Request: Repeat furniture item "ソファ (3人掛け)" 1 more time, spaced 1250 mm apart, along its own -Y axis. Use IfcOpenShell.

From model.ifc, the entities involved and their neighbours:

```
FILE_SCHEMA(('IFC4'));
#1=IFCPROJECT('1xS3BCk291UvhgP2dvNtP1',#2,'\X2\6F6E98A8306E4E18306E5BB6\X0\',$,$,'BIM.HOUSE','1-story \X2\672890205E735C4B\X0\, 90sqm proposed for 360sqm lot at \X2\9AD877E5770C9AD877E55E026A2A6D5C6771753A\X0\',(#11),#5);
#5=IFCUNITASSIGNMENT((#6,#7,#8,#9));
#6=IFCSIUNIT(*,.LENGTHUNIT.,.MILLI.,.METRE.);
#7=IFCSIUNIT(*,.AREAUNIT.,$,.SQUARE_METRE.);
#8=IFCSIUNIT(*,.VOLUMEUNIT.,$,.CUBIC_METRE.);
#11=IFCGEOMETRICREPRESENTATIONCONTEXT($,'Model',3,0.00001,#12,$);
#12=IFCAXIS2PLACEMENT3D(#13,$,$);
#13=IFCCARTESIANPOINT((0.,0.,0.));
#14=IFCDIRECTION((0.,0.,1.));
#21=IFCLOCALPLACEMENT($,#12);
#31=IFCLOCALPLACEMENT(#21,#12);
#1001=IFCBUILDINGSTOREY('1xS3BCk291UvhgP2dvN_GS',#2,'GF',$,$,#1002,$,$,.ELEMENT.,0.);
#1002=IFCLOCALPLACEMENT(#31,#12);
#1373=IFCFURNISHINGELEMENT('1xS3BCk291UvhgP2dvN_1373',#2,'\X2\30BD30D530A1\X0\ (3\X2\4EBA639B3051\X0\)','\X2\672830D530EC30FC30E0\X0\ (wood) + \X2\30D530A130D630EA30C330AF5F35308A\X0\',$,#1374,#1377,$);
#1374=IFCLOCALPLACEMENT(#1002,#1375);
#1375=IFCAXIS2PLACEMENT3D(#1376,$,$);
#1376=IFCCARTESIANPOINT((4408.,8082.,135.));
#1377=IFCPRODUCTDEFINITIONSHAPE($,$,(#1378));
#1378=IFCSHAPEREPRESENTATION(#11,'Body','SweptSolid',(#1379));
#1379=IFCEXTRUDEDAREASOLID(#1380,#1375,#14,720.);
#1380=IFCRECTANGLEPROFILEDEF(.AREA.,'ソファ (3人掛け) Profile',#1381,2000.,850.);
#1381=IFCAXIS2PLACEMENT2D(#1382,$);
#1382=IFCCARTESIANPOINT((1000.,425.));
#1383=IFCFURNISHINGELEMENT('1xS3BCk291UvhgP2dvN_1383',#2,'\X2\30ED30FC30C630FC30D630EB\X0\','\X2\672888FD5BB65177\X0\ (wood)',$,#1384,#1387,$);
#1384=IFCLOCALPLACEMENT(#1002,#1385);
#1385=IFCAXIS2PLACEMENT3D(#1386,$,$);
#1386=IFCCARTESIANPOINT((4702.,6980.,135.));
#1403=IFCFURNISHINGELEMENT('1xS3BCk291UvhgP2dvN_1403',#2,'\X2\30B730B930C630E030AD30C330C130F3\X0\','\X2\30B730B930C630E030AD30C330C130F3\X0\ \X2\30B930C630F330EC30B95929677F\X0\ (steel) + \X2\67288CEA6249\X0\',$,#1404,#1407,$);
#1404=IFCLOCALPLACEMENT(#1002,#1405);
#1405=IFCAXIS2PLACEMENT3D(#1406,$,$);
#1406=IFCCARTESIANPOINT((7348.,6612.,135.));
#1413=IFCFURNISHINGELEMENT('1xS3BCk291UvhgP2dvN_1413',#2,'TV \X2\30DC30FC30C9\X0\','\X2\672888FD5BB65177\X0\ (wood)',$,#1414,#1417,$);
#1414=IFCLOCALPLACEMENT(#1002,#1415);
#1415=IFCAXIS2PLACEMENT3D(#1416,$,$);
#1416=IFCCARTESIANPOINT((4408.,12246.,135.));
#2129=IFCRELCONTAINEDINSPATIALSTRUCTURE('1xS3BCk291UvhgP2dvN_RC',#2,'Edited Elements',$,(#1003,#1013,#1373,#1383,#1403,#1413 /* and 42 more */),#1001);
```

```python
import ifcopenshell
import ifcopenshell.api.geometry
import ifcopenshell.api.root
import ifcopenshell.util.element
import ifcopenshell.util.placement
import ifcopenshell.util.unit

model = ifcopenshell.open("model.ifc")
unit_scale = ifcopenshell.util.unit.calculate_unit_scale(model)


def reuse_history(source, copy):
    """copy_class also copies each property set's owner history, people and application; keep the originals."""
    for rel in copy.IsDefinedBy:
        if rel.is_a("IfcRelDefinesByProperties") and (history := rel.RelatingPropertyDefinition.OwnerHistory):
            rel.RelatingPropertyDefinition.OwnerHistory = source.OwnerHistory
            ifcopenshell.util.element.remove_deep2(model, history)


source = model.by_guid("1xS3BCk291UvhgP2dvN_1373")
base = ifcopenshell.util.placement.get_local_placement(source.ObjectPlacement)
step = -base[:3, 1] * 1.25 / unit_scale

for i in range(1, 2):
    copy = ifcopenshell.api.root.copy_class(model, product=source)
    copy.Representation = ifcopenshell.util.element.copy_deep(
        model, source.Representation, exclude=["IfcGeometricRepresentationContext", "IfcRepresentationMap"]
    )
    reuse_history(source, copy)
    matrix = base.copy()
    matrix[:3, 3] += i * step
    print("added at", matrix[:3, 3].round(3) + 0.0)
    ifcopenshell.api.geometry.edit_object_placement(model, product=copy, matrix=matrix, is_si=False)

model.write("model_v2.ifc")
```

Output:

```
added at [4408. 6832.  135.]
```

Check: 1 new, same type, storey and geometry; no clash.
